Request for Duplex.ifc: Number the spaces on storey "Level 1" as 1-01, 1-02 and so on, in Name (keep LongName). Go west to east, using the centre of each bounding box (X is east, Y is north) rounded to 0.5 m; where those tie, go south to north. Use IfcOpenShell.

First a look at what the model holds.

```python
import ifcopenshell
import ifcopenshell.util.element
import ifcopenshell.util.placement

model = ifcopenshell.open("Duplex.ifc")
print(model.schema)
storey = next(s for s in model.by_type("IfcBuildingStorey") if s.Name == "Level 1")
spaces = [e for e in ifcopenshell.util.element.get_decomposition(storey) if e.is_a("IfcSpace")]
for e in sorted(spaces, key=lambda e: e.id()):
    origin = ifcopenshell.util.placement.get_local_placement(e.ObjectPlacement)[:3, 3]
    print(e.id(), e.Name, e.LongName, origin.round(2) + 0.0, sep=" | ")
```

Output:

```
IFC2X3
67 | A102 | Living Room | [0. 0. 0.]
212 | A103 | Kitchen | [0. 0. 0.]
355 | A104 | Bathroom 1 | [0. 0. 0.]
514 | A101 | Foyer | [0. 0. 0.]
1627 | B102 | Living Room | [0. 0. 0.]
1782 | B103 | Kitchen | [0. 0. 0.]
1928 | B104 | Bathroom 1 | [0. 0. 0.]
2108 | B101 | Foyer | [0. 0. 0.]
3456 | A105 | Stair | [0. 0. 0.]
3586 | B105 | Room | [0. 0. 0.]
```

```python
import ifcopenshell
import ifcopenshell.geom
import ifcopenshell.util.element
import ifcopenshell.util.shape

model = ifcopenshell.open("Duplex.ifc")
settings = ifcopenshell.geom.settings()
settings.set("use-world-coords", True)


def centre(element):
    shape = ifcopenshell.geom.create_shape(settings, element)
    return ifcopenshell.util.shape.get_bbox_centroid(shape.geometry)


storey = next(s for s in model.by_type("IfcBuildingStorey") if s.Name == "Level 1")
spaces = [e for e in ifcopenshell.util.element.get_decomposition(storey) if e.is_a("IfcSpace")]

# Insertion points can sit at a corner or the storey origin, so sort by the geometry (in metres).
centres = {e: centre(e) for e in spaces}
spaces.sort(key=lambda e: (round(centres[e][0] / 0.5), centres[e][1]))

for i, e in enumerate(spaces, start=1):
    number = f"1-{i:02d}"
    e.Name = number
    print(e.id(), number)

model.write("Duplex_rev.ifc")
```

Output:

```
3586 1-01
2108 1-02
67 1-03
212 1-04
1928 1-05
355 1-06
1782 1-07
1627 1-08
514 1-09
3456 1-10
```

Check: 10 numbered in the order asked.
